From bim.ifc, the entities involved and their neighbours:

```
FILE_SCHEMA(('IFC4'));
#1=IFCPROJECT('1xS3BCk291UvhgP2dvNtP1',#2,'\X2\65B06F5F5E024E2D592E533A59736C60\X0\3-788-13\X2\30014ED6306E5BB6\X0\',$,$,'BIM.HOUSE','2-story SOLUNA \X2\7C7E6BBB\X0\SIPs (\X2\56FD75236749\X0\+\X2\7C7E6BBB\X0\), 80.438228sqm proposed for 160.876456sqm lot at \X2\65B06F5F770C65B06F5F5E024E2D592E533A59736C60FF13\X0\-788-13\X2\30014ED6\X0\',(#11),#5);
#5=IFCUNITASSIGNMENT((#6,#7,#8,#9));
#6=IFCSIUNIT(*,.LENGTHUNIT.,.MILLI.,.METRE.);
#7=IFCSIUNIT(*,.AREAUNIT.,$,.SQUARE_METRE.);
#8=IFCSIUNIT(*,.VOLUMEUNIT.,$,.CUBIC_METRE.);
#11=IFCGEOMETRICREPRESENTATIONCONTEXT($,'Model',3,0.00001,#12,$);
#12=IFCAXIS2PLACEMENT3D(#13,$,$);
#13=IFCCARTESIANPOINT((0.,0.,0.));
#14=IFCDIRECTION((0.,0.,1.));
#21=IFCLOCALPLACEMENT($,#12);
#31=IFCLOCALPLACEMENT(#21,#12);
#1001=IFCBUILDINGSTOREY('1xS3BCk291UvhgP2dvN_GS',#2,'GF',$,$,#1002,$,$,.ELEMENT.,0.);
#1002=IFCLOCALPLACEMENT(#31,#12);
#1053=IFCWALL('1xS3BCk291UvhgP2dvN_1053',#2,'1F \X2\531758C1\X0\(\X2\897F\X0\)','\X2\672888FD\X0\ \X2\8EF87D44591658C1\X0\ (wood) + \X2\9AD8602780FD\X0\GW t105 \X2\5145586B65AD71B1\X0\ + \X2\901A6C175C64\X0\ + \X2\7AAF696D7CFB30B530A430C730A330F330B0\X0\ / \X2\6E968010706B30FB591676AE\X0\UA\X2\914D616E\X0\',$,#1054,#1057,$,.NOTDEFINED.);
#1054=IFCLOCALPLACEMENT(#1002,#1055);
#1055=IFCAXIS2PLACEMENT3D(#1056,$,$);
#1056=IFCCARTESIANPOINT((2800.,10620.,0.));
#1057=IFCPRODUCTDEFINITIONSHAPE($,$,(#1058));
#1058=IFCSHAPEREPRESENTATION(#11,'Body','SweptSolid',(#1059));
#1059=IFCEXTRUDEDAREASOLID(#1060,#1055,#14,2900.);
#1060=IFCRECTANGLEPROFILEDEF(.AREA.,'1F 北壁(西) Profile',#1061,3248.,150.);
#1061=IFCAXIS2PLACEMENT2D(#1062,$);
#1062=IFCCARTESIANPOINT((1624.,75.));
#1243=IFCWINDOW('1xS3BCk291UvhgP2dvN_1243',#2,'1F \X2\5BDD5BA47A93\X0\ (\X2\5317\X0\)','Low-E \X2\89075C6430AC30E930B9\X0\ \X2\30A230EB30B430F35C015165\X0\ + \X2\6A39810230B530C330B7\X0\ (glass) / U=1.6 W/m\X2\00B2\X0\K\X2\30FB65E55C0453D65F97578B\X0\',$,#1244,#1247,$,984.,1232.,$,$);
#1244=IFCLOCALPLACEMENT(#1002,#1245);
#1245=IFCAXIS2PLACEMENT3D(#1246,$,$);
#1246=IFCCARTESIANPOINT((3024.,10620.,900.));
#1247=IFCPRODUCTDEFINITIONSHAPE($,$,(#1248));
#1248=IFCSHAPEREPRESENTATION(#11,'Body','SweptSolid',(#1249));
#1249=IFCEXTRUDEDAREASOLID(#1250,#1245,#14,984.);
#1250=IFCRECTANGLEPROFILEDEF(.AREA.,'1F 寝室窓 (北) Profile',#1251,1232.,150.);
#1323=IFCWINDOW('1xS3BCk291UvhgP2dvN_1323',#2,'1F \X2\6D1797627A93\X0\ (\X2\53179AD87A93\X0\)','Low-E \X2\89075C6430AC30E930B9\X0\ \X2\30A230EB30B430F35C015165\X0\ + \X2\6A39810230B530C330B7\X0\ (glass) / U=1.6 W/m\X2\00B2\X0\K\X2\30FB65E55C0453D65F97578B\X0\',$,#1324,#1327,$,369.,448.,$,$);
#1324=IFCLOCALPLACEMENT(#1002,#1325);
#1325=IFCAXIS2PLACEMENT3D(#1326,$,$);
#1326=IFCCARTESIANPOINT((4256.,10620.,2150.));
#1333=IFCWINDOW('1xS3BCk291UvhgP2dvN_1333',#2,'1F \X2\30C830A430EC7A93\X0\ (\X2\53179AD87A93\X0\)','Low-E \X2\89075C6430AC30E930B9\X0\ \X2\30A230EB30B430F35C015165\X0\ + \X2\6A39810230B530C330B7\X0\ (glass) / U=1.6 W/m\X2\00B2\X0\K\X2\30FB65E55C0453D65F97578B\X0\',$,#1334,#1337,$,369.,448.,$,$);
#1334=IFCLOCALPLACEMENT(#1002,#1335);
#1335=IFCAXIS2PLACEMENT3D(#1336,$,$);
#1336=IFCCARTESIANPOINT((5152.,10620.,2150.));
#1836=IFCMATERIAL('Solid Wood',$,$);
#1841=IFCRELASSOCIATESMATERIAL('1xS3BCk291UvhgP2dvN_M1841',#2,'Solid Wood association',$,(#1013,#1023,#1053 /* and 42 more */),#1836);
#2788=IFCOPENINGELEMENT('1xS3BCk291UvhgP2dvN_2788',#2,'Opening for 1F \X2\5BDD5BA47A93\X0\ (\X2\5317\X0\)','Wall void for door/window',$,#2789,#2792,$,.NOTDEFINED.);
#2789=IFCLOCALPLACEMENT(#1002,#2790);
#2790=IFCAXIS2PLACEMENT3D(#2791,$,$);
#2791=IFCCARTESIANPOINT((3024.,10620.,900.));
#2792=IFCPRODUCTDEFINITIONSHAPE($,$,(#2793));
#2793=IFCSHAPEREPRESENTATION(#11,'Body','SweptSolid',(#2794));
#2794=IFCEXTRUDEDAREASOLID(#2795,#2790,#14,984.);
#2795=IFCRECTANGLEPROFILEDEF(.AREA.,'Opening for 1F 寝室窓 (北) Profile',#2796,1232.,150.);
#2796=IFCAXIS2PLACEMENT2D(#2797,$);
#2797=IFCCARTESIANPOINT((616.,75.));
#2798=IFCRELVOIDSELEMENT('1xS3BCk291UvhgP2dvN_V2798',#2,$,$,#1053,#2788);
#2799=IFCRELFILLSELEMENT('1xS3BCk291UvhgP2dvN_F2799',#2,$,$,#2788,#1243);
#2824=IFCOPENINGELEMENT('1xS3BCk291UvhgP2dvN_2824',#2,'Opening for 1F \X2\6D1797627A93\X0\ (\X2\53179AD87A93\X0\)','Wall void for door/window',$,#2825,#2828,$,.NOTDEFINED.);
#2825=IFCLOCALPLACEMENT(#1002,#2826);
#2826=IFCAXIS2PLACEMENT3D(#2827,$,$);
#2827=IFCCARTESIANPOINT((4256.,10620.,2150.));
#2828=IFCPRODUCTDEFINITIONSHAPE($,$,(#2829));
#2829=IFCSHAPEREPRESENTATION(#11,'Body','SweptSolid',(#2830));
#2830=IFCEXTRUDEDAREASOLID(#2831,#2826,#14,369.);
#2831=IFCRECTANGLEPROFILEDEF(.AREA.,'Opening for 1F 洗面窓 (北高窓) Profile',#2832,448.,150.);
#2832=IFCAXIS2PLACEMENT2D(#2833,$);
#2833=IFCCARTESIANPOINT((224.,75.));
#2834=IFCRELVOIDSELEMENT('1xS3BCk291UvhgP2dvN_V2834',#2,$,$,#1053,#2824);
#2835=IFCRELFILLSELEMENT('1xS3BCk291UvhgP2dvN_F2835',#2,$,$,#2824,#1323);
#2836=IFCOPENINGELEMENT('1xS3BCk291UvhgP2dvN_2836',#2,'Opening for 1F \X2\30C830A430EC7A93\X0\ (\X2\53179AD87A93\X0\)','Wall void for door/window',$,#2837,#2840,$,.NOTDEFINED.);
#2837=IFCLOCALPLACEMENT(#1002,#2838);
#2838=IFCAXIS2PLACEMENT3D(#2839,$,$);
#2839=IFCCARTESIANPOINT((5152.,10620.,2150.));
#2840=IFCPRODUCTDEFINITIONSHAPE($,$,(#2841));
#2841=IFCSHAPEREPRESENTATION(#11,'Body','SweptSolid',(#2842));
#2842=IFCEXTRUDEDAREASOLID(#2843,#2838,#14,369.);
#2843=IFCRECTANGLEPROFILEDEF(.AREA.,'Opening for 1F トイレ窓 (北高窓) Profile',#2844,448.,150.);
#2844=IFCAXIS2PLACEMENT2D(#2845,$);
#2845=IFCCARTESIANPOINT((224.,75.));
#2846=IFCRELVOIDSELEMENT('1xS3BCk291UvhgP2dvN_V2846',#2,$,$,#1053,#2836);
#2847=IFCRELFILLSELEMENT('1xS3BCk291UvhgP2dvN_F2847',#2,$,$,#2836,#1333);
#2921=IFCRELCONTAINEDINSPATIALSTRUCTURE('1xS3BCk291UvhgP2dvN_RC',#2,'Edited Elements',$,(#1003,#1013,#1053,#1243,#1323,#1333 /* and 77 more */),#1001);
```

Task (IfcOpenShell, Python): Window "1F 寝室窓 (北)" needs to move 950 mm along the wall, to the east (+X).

```python
import ifcopenshell
import ifcopenshell.api.geometry
import ifcopenshell.util.placement

model = ifcopenshell.open("bim.ifc")

window = model.by_guid("1xS3BCk291UvhgP2dvN_1243")
opening = window.FillsVoids[0].RelatingOpeningElement
wall = opening.VoidsElements[0].RelatingBuildingElement

wall_matrix = ifcopenshell.util.placement.get_local_placement(wall.ObjectPlacement)
shift = wall_matrix[:3, 0] * 950.0
before = ifcopenshell.util.placement.get_local_placement(window.ObjectPlacement)[:3, 3].copy()

# The window is not placed relative to its opening, so move both.
for product in (opening, window):
    matrix = ifcopenshell.util.placement.get_local_placement(product.ObjectPlacement)
    matrix[:3, 3] += shift
    ifcopenshell.api.geometry.edit_object_placement(model, product=product, matrix=matrix, is_si=False)

after = ifcopenshell.util.placement.get_local_placement(window.ObjectPlacement)[:3, 3]
print("window moved by", (after - before).round(3) + 0.0)

model.write("bim_rev.ifc")
```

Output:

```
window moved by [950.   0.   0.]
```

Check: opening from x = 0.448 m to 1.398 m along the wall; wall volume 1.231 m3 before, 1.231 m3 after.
